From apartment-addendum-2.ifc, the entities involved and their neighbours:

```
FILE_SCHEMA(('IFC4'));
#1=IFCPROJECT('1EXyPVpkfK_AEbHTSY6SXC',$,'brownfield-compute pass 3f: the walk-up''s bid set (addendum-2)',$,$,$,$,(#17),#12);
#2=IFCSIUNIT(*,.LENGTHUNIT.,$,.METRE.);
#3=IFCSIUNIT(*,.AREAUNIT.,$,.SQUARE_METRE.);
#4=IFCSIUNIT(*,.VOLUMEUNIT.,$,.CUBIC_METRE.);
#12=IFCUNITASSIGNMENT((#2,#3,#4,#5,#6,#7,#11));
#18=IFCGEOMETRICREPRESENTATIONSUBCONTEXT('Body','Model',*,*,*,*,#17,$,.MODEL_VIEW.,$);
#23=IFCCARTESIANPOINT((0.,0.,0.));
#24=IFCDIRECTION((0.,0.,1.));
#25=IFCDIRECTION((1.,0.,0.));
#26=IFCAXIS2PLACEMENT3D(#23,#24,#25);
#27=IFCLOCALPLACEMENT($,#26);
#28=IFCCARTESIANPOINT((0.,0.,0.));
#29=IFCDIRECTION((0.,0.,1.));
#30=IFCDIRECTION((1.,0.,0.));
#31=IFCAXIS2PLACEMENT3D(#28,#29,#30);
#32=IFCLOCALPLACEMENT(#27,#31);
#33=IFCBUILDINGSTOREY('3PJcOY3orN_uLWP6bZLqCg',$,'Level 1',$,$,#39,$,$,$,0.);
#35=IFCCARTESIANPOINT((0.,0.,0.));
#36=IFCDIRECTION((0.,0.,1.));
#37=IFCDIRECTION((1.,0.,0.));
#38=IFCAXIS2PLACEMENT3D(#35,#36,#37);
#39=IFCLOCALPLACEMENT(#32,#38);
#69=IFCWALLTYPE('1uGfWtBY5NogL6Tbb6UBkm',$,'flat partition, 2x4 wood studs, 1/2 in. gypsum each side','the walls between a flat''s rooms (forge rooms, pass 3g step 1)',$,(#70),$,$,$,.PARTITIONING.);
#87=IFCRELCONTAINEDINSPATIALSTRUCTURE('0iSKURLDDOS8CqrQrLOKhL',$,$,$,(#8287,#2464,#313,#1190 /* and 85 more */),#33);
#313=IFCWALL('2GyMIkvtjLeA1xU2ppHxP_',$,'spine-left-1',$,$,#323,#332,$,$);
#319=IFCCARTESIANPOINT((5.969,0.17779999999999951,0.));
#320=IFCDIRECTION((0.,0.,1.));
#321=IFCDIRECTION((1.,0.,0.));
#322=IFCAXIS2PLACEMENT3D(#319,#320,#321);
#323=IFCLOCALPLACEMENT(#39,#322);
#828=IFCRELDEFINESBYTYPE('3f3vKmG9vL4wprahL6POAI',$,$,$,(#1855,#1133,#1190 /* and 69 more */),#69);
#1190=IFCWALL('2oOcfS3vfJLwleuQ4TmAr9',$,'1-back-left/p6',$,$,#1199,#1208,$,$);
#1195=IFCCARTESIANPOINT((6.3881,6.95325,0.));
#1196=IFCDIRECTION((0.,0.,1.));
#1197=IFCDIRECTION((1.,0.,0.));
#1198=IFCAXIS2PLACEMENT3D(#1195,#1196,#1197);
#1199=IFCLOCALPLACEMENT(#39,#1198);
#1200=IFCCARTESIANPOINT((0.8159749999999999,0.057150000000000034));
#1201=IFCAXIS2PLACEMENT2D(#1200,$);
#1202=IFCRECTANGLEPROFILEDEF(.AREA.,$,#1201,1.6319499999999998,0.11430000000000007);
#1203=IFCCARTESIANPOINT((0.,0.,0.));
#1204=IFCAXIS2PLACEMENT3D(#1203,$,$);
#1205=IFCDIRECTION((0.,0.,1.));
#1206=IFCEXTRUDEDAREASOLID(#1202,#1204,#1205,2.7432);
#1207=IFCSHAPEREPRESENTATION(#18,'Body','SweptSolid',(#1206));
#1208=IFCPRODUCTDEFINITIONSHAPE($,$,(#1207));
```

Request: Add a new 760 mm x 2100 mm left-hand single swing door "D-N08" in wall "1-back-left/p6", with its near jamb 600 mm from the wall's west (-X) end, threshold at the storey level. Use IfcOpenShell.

```python
import numpy as np
import ifcopenshell
import ifcopenshell.api.feature
import ifcopenshell.api.geometry
import ifcopenshell.api.root
import ifcopenshell.api.spatial
import ifcopenshell.geom
import ifcopenshell.util.element
import ifcopenshell.util.placement
import ifcopenshell.util.representation
import ifcopenshell.util.shape
import ifcopenshell.util.unit

model = ifcopenshell.open("apartment-addendum-2.ifc")
unit_scale = ifcopenshell.util.unit.calculate_unit_scale(model)
settings = ifcopenshell.geom.settings()


def volume(element):
    """Net volume in cubic metres, openings subtracted."""
    shape = ifcopenshell.geom.create_shape(settings, element)
    return ifcopenshell.util.shape.get_volume(shape.geometry)


wall = model.by_guid("2oOcfS3vfJLwleuQ4TmAr9")
storey = ifcopenshell.util.element.get_container(wall, ifc_class="IfcBuildingStorey")
context = ifcopenshell.util.representation.get_context(model, "Model", "Body", "MODEL_VIEW")
before = volume(wall)

width, height, from_end, sill = 0.76, 2.1, 0.6, 0.0  # metres

# The wall runs along its own X axis, and the end named is its -X end.
wall_shape = ifcopenshell.geom.create_shape(settings, wall)
x, y, z = ifcopenshell.util.shape.get_vertices(wall_shape.geometry).T
start = x.min() + from_end
face, thickness = float(y.min()), float(y.max() - y.min())
wall_matrix = ifcopenshell.util.placement.get_local_placement(wall.ObjectPlacement)
level = ifcopenshell.util.placement.get_local_placement(storey.ObjectPlacement)[2, 3]


def in_wall(x, y):
    """Placement at x, y metres in the wall's axes, at sill height."""
    matrix = wall_matrix.copy()
    matrix[:, 3] = wall_matrix @ np.array([x / unit_scale, y / unit_scale, 0.0, 1.0])
    matrix[2, 3] = level + sill / unit_scale
    return matrix


# Opening: a box that overshoots both wall faces by 50 mm.
opening = ifcopenshell.api.root.create_entity(model, ifc_class="IfcOpeningElement", predefined_type="OPENING")
box = ifcopenshell.api.geometry.add_wall_representation(
    model, context=context, length=width, height=height, thickness=thickness + 0.1
)
ifcopenshell.api.geometry.assign_representation(model, product=opening, representation=box)
ifcopenshell.api.geometry.edit_object_placement(model, product=opening, matrix=in_wall(start, face - 0.05), is_si=False)
ifcopenshell.api.feature.add_feature(model, feature=opening, element=wall)

door = ifcopenshell.api.root.create_entity(model, ifc_class="IfcDoor", name="D-N08", predefined_type="DOOR")
door.OverallWidth, door.OverallHeight = width / unit_scale, height / unit_scale
door.OperationType = "SINGLE_SWING_LEFT"
body = ifcopenshell.api.geometry.add_door_representation(
    model,
    context=context,
    overall_width=door.OverallWidth,
    overall_height=door.OverallHeight,
    operation_type="SINGLE_SWING_LEFT",
    lining_properties={"LiningDepth": thickness / unit_scale, "ThresholdDepth": thickness / unit_scale},
)
ifcopenshell.api.geometry.assign_representation(model, product=door, representation=body)
ifcopenshell.api.spatial.assign_container(model, products=[door], relating_structure=storey)
ifcopenshell.api.feature.add_filling(model, opening=opening, element=door)

# The lining spans the wall, so the door starts at the wall face.
ifcopenshell.api.geometry.edit_object_placement(model, product=door, matrix=in_wall(start, face), is_si=False)

after = volume(wall)

print(f"wall volume {before:.3f} -> {after:.3f} m3")

model.write("apartment-addendum-2_rev.ifc")
```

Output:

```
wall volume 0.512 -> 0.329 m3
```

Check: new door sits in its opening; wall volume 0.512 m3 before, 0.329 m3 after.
